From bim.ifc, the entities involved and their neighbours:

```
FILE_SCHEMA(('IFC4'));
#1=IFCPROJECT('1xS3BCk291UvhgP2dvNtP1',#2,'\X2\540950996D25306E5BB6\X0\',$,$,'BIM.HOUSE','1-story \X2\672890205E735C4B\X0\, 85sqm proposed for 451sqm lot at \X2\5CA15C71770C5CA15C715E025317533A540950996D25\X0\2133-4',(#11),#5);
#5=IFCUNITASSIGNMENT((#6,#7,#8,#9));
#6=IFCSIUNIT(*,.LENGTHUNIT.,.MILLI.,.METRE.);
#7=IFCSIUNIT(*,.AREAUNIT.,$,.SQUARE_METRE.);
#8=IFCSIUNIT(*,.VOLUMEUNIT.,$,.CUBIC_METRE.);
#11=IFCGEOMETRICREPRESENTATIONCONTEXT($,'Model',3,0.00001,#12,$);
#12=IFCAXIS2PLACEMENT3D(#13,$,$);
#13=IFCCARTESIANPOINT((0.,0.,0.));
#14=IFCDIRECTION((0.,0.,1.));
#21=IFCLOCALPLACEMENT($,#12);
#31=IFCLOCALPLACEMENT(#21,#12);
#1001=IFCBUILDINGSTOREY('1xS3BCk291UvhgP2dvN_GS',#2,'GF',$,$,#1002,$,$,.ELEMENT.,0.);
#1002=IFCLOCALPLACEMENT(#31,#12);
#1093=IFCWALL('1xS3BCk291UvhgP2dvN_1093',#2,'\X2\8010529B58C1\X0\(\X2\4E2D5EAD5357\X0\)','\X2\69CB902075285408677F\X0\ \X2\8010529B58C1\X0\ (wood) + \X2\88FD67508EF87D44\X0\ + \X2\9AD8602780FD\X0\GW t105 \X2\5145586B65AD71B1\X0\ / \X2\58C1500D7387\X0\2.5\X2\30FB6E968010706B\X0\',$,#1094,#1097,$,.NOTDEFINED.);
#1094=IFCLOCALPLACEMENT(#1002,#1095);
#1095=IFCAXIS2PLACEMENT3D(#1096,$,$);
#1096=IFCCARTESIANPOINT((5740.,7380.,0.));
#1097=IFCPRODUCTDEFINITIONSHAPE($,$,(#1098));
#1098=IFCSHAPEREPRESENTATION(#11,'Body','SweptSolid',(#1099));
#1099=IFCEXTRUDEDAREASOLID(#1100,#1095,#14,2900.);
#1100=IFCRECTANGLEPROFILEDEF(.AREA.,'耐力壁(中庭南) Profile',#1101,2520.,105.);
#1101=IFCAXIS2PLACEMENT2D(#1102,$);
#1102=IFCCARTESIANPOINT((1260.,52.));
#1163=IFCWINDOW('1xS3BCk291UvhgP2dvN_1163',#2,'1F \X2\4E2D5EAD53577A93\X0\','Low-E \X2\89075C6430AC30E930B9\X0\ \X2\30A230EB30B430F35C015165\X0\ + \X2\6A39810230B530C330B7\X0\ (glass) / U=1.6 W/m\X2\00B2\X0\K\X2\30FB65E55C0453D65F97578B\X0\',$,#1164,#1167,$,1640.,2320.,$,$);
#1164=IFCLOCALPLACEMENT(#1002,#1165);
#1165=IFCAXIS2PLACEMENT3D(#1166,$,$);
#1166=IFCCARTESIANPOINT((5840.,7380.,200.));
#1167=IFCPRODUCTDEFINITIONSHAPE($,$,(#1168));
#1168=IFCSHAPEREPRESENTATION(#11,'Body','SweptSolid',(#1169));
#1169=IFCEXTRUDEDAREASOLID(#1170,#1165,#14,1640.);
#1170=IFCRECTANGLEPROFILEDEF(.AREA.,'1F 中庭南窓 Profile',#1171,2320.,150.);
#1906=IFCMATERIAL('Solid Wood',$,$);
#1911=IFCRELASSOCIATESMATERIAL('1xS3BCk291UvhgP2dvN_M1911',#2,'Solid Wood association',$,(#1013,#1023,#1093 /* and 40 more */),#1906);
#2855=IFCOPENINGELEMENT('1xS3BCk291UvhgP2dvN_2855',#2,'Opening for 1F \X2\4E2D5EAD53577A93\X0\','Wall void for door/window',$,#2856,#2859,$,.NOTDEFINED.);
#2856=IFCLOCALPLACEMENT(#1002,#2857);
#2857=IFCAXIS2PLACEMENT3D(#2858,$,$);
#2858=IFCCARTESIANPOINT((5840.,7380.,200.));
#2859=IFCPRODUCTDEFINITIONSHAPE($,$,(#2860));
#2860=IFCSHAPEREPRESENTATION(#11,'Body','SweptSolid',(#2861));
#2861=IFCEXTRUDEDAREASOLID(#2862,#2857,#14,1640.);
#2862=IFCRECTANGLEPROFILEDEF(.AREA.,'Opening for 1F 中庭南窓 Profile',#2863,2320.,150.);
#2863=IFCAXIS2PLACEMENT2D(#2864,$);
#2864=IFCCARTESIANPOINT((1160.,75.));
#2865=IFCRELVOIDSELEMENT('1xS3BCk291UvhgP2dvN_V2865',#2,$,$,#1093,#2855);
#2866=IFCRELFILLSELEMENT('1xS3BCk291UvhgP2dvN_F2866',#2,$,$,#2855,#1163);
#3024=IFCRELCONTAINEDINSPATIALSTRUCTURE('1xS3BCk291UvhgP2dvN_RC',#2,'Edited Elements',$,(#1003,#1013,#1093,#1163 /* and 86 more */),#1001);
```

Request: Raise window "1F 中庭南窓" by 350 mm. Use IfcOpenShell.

```python
import numpy as np
import ifcopenshell
import ifcopenshell.api.geometry
import ifcopenshell.util.placement
import ifcopenshell.util.unit

model = ifcopenshell.open("bim.ifc")
unit_scale = ifcopenshell.util.unit.calculate_unit_scale(model)

window = model.by_id(1163)
opening = window.FillsVoids[0].RelatingOpeningElement
dz = 0.35 / unit_scale

shift = np.array([0.0, 0.0, dz])
# The window is not placed relative to its opening, so move both.
for product in (opening, window):
    matrix = ifcopenshell.util.placement.get_local_placement(product.ObjectPlacement)
    matrix[:3, 3] += shift
    ifcopenshell.api.geometry.edit_object_placement(model, product=product, matrix=matrix, is_si=False)

print(f"moved by {dz * unit_scale:+.3f} m")

model.write("bim_updated.ifc")
```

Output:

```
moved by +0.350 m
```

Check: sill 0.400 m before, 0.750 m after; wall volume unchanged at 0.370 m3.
